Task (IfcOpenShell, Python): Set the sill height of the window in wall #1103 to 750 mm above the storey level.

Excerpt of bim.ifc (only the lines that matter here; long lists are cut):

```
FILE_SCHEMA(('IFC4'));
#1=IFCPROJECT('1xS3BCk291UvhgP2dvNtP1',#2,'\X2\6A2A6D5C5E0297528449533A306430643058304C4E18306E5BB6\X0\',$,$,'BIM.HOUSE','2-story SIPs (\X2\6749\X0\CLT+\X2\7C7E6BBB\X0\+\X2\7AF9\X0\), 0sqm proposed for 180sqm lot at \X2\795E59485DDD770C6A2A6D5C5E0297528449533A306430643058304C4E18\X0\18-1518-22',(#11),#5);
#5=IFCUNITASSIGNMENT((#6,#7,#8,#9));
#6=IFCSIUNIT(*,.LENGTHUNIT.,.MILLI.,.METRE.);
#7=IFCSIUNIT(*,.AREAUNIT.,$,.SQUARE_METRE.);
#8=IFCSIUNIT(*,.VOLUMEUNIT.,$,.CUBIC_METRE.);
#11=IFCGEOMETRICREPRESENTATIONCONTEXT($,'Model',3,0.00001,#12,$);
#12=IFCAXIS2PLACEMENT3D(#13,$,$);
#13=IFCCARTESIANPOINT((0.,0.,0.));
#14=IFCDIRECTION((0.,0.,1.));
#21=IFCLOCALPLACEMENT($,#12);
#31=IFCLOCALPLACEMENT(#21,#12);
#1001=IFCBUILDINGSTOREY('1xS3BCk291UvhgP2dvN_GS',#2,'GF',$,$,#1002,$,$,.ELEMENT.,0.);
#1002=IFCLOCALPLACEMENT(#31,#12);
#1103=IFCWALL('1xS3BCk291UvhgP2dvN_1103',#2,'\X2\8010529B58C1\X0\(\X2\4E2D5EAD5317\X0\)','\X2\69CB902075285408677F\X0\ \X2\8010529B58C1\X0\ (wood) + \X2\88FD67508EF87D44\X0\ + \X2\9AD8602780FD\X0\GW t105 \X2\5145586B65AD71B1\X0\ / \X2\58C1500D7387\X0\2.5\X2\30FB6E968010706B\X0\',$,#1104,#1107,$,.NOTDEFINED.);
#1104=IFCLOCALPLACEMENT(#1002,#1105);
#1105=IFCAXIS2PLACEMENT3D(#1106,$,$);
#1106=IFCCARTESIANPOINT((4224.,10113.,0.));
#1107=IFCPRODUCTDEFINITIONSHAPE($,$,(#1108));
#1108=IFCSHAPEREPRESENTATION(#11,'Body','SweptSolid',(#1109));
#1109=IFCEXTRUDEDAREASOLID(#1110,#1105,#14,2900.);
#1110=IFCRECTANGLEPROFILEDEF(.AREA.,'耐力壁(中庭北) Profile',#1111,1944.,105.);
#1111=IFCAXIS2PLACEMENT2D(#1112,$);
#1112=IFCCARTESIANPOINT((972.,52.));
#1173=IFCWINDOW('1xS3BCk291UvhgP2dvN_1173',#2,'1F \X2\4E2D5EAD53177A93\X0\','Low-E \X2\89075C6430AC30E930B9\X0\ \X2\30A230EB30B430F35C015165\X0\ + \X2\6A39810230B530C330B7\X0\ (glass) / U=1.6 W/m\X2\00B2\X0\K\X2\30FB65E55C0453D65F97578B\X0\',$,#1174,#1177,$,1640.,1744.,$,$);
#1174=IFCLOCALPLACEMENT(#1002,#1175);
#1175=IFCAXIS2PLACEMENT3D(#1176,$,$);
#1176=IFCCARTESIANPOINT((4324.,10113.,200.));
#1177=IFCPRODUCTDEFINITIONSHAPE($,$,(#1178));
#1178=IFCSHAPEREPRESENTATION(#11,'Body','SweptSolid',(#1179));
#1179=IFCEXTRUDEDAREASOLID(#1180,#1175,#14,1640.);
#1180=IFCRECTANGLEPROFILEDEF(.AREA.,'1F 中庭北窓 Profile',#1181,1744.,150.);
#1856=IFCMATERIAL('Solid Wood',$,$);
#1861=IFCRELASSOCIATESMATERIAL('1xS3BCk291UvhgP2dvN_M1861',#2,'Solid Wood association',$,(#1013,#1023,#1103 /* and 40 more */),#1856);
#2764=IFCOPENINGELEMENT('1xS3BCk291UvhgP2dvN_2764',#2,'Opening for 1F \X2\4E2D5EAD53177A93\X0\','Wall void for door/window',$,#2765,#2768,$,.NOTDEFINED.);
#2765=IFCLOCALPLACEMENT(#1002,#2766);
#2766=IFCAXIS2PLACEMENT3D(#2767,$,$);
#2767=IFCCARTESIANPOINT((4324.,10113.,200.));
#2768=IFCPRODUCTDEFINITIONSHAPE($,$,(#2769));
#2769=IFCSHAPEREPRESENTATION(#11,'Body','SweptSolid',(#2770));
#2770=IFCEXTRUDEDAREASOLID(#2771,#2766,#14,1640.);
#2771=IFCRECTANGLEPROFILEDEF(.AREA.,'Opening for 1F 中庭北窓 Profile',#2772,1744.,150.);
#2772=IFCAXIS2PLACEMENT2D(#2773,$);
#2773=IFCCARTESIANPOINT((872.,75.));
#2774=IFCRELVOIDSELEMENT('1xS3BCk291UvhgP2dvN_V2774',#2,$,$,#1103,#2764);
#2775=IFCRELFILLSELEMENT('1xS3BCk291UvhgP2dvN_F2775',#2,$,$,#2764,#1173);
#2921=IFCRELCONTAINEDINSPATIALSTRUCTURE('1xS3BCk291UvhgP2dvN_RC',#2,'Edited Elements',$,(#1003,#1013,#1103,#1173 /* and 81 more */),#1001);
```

```python
import numpy as np
import ifcopenshell
import ifcopenshell.api.geometry
import ifcopenshell.geom
import ifcopenshell.util.element
import ifcopenshell.util.placement
import ifcopenshell.util.shape
import ifcopenshell.util.unit

model = ifcopenshell.open("bim.ifc")
unit_scale = ifcopenshell.util.unit.calculate_unit_scale(model)

window = model.by_guid("1xS3BCk291UvhgP2dvN_1173")
opening = window.FillsVoids[0].RelatingOpeningElement
storey = ifcopenshell.util.element.get_container(window, ifc_class="IfcBuildingStorey")
level = ifcopenshell.util.placement.get_local_placement(storey.ObjectPlacement)[2, 3]

# The opening's origin need not be at the sill, so measure its lowest point.
shape = ifcopenshell.geom.create_shape(ifcopenshell.geom.settings(), opening)
bottom = ifcopenshell.util.shape.get_shape_bottom_elevation(shape, shape.geometry) / unit_scale
dz = level + 0.75 / unit_scale - bottom

shift = np.array([0.0, 0.0, dz])
# The window is not placed relative to its opening, so move both.
for product in (opening, window):
    matrix = ifcopenshell.util.placement.get_local_placement(product.ObjectPlacement)
    matrix[:3, 3] += shift
    ifcopenshell.api.geometry.edit_object_placement(model, product=product, matrix=matrix, is_si=False)

print(f"moved by {dz * unit_scale:+.3f} m")

model.write("bim_rev.ifc")
```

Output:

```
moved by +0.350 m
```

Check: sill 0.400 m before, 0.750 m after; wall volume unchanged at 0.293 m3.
